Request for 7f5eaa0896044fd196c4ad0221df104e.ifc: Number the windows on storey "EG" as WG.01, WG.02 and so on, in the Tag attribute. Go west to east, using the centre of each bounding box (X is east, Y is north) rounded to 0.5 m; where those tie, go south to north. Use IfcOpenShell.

First a look at what the model holds.

```python
import ifcopenshell
import ifcopenshell.util.element
import ifcopenshell.util.placement

model = ifcopenshell.open("7f5eaa0896044fd196c4ad0221df104e.ifc")
print(model.schema)
storey = next(s for s in model.by_type("IfcBuildingStorey") if s.Name == "EG")
windows = [e for e in ifcopenshell.util.element.get_decomposition(storey) if e.is_a("IfcWindow")]
for e in sorted(windows, key=lambda e: e.id()):
    origin = ifcopenshell.util.placement.get_local_placement(e.ObjectPlacement)[:3, 3]
    print(e.id(), e.Tag, e.Name, origin.round(2) + 0.0, sep=" | ")
```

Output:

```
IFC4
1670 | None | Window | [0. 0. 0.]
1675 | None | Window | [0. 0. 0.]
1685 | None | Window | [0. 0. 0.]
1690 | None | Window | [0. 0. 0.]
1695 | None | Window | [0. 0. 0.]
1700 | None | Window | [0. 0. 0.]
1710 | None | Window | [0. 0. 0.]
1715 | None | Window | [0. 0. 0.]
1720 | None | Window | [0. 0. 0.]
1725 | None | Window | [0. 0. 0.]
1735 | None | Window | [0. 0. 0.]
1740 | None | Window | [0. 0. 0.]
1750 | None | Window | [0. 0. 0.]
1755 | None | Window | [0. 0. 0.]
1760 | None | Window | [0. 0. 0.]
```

```python
import ifcopenshell
import ifcopenshell.geom
import ifcopenshell.util.element
import ifcopenshell.util.shape

model = ifcopenshell.open("7f5eaa0896044fd196c4ad0221df104e.ifc")
settings = ifcopenshell.geom.settings()
settings.set("use-world-coords", True)


def centre(element):
    shape = ifcopenshell.geom.create_shape(settings, element)
    return ifcopenshell.util.shape.get_bbox_centroid(shape.geometry)


storey = next(s for s in model.by_type("IfcBuildingStorey") if s.Name == "EG")
windows = [e for e in ifcopenshell.util.element.get_decomposition(storey) if e.is_a("IfcWindow")]

# Insertion points can sit at a corner or the storey origin, so sort by the geometry (in metres).
centres = {e: centre(e) for e in windows}
windows.sort(key=lambda e: (round(centres[e][0] / 0.5), centres[e][1]))

for i, e in enumerate(windows, start=1):
    number = f"WG.{i:02d}"
    e.Tag = number
    print(e.id(), number)

model.write("7f5eaa0896044fd196c4ad0221df104e_updated.ifc")
```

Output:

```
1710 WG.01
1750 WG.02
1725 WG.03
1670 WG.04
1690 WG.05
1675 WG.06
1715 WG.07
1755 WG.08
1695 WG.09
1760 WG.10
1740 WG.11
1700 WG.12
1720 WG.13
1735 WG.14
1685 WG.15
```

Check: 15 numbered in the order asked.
